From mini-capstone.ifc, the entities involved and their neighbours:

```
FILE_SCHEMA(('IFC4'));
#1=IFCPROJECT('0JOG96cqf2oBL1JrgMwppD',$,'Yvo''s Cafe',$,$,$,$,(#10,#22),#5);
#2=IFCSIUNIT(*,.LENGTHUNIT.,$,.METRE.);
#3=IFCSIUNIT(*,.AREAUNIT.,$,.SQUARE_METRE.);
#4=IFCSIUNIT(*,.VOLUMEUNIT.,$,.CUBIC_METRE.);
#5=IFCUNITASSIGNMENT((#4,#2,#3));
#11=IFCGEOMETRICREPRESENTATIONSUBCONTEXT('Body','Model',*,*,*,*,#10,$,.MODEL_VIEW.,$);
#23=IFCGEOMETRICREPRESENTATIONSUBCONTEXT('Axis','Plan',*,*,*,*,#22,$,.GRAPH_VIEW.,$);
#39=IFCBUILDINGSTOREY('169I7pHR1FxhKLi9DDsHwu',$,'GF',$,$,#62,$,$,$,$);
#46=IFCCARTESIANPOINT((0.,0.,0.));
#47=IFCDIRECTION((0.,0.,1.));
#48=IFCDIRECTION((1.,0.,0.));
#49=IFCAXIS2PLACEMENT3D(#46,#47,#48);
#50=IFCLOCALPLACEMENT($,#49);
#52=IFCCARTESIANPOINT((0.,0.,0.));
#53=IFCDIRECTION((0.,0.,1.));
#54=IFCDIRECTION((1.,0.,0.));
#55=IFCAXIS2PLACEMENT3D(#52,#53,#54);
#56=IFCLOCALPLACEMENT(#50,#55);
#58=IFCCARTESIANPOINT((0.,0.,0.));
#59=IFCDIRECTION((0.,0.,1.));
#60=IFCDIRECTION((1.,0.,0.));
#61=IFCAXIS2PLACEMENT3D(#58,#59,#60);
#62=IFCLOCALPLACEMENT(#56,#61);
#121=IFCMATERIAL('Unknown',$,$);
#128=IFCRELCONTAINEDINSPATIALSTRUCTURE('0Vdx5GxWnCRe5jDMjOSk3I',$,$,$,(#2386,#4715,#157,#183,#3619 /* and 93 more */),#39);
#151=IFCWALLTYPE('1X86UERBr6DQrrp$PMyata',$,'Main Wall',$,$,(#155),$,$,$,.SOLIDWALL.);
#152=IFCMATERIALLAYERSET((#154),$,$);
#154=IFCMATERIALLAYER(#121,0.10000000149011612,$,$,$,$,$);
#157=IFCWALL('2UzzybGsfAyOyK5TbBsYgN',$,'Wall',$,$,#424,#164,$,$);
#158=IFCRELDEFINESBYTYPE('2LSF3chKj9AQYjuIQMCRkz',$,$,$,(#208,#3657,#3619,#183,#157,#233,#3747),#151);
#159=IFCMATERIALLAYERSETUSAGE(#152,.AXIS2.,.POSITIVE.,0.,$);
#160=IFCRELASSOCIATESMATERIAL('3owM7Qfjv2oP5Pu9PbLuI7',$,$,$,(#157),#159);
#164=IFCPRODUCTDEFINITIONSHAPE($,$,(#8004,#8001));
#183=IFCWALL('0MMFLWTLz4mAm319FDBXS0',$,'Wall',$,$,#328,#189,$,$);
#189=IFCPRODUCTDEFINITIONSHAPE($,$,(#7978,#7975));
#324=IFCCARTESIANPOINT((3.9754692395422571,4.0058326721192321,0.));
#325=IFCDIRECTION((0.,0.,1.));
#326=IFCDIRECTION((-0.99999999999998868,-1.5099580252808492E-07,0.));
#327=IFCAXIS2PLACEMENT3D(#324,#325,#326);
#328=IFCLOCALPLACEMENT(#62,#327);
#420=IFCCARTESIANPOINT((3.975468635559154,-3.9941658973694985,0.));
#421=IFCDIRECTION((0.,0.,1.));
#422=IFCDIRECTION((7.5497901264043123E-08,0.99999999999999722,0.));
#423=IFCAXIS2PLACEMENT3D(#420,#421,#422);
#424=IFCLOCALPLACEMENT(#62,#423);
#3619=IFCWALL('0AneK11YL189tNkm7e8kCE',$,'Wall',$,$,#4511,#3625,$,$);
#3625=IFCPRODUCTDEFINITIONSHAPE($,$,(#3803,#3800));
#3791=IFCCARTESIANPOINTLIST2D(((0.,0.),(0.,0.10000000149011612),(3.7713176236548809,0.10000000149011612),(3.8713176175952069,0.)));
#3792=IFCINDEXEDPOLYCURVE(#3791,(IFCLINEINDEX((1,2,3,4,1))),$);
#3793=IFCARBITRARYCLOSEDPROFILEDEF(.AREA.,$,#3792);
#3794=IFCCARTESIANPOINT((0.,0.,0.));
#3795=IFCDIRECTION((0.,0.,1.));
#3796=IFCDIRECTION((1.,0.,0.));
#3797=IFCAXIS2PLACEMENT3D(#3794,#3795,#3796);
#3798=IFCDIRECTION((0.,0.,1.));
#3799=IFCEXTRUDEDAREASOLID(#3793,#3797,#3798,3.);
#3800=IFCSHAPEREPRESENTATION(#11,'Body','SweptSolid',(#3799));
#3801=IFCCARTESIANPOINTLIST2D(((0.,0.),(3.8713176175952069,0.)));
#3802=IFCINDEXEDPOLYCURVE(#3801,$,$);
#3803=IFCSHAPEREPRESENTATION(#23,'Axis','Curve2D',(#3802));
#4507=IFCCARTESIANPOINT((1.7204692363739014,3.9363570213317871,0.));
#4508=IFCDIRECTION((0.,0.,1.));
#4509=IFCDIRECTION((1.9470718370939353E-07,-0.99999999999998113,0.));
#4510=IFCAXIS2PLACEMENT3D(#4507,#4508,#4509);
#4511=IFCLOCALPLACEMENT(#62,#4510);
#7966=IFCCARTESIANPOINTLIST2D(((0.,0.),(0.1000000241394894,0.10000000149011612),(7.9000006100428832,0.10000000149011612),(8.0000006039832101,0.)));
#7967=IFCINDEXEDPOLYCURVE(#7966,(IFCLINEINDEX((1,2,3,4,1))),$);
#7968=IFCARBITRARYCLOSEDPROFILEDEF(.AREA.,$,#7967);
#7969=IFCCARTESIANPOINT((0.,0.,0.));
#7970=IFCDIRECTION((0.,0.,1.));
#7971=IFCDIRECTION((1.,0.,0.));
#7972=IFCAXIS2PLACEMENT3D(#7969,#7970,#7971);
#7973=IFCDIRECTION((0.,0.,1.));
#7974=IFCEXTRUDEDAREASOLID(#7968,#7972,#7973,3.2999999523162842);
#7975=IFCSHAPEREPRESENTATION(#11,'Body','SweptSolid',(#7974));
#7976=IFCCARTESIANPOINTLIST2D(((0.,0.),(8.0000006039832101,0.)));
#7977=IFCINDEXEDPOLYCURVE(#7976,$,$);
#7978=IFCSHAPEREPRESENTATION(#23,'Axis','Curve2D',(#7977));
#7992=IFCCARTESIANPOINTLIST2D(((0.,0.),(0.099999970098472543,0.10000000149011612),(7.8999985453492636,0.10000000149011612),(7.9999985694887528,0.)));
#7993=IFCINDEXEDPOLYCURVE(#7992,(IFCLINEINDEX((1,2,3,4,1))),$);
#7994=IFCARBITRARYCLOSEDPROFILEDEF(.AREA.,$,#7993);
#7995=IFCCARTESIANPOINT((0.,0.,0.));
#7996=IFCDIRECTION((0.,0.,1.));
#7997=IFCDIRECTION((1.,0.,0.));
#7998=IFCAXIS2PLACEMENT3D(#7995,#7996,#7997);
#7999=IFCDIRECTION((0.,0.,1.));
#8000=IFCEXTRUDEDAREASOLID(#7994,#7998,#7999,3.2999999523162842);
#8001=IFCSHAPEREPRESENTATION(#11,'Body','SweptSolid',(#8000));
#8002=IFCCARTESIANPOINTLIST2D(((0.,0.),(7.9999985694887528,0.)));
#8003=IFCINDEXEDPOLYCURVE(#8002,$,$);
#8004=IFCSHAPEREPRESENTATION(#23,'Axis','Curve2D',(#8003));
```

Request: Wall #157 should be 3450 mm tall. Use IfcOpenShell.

```python
import ifcopenshell
import ifcopenshell.geom
import ifcopenshell.util.representation
import ifcopenshell.util.shape

model = ifcopenshell.open("mini-capstone.ifc")
settings = ifcopenshell.geom.settings()


def volume(element):
    """Net volume in cubic metres, openings subtracted."""
    shape = ifcopenshell.geom.create_shape(settings, element)
    return ifcopenshell.util.shape.get_volume(shape.geometry)


wall = model.by_guid("2UzzybGsfAyOyK5TbBsYgN")
before = volume(wall)

body = ifcopenshell.util.representation.get_representation(wall, "Model", "Body")
solid = body.Items[0]
old_height = solid.Depth
solid.Depth = 3.45
after = volume(wall)

print(f"height {old_height:g} -> {solid.Depth:g}, volume {before:.3f} -> {after:.3f} m3")

model.write("mini-capstone_edited.ifc")
```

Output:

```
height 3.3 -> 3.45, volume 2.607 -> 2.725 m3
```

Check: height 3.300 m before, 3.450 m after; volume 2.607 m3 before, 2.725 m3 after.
